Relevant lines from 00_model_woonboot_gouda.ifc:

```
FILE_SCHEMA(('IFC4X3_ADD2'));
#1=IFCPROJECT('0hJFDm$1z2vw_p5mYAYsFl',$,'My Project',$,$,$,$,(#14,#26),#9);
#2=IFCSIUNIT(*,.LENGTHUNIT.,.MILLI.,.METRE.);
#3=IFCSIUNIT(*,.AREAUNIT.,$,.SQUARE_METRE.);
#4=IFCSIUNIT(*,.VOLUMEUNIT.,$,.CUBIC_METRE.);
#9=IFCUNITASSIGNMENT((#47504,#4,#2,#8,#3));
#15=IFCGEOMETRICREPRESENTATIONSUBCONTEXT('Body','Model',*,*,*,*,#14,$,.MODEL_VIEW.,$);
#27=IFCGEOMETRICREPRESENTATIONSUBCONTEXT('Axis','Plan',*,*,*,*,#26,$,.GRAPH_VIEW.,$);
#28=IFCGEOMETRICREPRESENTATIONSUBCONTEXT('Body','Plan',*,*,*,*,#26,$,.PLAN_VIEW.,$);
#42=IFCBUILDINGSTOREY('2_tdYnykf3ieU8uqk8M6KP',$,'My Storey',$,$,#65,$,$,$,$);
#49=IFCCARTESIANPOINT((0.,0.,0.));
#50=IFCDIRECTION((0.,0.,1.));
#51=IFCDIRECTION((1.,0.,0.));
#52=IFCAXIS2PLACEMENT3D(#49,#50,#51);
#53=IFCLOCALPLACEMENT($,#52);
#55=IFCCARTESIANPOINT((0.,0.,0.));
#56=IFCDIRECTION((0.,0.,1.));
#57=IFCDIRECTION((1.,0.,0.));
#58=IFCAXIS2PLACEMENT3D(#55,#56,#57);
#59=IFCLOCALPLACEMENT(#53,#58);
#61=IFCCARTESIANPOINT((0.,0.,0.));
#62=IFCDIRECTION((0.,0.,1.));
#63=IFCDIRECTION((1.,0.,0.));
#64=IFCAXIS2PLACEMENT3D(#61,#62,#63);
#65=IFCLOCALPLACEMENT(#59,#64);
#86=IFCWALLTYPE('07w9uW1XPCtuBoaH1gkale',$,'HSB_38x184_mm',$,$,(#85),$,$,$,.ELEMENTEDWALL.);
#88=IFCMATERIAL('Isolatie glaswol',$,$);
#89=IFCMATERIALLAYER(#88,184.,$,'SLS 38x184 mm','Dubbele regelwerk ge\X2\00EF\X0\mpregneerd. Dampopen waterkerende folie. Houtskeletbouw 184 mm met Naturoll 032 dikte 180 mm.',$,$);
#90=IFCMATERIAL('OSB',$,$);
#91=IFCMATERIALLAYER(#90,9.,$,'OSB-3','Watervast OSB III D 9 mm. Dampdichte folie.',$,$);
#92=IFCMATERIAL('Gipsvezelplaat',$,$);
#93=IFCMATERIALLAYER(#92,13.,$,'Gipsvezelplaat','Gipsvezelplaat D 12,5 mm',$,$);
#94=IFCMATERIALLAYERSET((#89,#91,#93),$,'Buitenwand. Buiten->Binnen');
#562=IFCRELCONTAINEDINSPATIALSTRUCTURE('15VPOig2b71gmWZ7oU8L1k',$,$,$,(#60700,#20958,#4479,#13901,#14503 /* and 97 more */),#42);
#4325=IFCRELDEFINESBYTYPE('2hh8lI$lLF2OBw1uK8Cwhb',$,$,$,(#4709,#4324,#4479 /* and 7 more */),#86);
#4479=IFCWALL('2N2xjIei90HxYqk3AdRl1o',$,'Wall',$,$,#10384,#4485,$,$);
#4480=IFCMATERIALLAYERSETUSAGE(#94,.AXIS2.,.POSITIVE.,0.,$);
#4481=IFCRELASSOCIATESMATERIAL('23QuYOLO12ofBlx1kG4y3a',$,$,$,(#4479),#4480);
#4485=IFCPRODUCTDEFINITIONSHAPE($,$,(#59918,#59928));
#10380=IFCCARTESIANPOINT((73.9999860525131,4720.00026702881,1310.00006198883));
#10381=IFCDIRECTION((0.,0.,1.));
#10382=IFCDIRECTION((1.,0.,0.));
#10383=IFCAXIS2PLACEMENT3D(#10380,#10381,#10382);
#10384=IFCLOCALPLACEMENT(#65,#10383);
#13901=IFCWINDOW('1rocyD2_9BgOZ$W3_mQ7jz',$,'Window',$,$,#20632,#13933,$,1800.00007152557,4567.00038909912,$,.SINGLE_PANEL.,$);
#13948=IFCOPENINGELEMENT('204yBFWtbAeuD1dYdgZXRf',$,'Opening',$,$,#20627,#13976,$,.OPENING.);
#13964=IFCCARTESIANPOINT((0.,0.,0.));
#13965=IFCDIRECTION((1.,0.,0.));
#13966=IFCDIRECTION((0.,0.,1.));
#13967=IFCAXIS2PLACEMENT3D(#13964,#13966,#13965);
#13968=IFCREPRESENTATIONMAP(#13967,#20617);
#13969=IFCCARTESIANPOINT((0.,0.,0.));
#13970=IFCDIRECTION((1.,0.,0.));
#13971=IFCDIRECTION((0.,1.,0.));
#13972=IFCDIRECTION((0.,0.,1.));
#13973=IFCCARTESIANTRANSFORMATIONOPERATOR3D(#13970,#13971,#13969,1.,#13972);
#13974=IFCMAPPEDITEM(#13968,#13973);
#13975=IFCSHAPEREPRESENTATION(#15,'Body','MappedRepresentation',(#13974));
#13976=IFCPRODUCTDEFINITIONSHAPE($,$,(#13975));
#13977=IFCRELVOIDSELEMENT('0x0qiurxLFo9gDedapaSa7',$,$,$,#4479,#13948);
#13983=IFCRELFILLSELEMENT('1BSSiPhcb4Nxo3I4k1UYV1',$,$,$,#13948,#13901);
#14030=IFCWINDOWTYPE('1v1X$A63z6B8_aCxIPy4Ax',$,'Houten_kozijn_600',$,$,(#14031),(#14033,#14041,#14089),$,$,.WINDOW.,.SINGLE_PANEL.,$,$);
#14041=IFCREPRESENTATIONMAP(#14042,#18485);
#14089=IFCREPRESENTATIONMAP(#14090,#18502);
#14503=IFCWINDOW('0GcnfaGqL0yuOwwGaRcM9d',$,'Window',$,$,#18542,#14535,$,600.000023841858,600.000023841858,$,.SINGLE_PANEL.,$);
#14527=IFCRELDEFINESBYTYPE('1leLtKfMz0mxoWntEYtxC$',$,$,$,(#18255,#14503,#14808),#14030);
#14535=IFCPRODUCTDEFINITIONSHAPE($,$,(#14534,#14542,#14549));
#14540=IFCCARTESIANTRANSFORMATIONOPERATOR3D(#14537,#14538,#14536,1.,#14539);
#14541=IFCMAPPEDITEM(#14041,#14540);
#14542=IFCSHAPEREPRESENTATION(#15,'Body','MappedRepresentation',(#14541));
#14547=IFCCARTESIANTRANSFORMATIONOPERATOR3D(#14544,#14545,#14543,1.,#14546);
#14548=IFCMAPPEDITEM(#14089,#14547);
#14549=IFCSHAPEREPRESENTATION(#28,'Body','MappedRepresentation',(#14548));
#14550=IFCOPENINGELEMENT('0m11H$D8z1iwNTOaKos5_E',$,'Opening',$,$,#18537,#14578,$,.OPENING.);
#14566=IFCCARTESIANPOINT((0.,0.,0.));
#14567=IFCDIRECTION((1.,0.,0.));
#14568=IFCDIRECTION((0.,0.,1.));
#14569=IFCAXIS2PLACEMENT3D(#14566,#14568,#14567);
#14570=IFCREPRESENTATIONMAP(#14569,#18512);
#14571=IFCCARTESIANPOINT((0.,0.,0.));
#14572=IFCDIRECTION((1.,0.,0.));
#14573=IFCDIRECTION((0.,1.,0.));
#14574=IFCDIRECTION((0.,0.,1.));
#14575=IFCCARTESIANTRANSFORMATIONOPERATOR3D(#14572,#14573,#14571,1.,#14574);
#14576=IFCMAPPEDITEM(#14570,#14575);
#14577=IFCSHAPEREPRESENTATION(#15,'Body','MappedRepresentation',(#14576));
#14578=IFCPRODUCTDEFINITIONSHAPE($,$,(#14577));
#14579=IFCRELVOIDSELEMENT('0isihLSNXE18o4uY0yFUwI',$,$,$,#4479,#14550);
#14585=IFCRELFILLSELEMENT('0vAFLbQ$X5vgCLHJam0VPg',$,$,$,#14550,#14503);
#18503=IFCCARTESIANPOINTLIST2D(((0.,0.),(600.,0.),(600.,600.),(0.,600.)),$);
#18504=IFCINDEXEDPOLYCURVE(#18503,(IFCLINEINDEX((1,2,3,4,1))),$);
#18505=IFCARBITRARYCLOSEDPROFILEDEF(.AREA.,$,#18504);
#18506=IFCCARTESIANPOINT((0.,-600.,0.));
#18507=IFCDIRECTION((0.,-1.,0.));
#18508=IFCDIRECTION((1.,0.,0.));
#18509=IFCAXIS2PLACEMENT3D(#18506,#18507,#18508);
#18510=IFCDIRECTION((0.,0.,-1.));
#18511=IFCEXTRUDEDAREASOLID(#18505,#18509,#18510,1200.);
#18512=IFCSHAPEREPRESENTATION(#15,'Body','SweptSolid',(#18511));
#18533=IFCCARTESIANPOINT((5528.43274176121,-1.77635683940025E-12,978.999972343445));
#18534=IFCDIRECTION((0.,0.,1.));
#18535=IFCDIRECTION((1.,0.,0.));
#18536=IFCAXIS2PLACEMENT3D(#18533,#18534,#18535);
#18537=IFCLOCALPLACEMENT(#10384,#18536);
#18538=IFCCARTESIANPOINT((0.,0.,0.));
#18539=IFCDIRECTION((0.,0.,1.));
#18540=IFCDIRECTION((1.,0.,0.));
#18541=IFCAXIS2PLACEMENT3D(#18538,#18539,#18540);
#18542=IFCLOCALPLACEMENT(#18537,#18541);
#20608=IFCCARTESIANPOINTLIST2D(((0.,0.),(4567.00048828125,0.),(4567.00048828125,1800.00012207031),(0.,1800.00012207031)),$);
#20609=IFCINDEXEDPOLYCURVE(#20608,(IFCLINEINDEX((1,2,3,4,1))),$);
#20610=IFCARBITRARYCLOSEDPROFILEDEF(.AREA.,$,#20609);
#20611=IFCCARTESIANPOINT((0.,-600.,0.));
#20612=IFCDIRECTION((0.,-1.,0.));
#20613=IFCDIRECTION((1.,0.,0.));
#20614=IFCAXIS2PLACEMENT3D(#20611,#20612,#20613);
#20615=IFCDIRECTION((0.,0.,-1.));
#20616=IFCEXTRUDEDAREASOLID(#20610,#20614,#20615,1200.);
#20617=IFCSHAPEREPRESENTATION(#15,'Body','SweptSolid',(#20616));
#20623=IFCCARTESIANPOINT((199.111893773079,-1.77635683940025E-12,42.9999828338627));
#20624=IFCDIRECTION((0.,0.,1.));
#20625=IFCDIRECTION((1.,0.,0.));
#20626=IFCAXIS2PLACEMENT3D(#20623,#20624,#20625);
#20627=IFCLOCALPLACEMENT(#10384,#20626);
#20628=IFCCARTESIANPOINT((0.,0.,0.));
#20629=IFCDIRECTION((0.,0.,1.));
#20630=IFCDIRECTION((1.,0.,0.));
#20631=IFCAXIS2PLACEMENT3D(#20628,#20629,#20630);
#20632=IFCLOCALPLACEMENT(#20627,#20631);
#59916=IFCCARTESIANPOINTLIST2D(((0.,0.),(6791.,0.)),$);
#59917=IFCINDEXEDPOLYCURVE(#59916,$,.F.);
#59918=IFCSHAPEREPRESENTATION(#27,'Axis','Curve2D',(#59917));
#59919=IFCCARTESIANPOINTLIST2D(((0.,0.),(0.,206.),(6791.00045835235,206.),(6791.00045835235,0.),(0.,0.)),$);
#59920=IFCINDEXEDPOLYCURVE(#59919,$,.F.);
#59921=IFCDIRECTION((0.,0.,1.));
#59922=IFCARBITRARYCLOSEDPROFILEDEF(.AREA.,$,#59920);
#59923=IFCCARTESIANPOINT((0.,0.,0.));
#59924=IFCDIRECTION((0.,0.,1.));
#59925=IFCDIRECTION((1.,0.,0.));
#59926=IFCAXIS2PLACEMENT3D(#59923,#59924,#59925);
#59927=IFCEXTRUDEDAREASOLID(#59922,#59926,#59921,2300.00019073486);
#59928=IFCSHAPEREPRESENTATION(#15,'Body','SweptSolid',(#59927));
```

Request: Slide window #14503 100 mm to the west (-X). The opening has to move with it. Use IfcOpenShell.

```python
import ifcopenshell
import ifcopenshell.api.geometry
import ifcopenshell.util.placement

model = ifcopenshell.open("00_model_woonboot_gouda.ifc")

window = model.by_guid("0GcnfaGqL0yuOwwGaRcM9d")
opening = window.FillsVoids[0].RelatingOpeningElement
wall = opening.VoidsElements[0].RelatingBuildingElement

wall_matrix = ifcopenshell.util.placement.get_local_placement(wall.ObjectPlacement)
shift = wall_matrix[:3, 0] * -100.0
before = ifcopenshell.util.placement.get_local_placement(window.ObjectPlacement)[:3, 3].copy()

# The window is placed relative to its opening, so it follows when the opening moves.
matrix = ifcopenshell.util.placement.get_local_placement(opening.ObjectPlacement)
matrix[:3, 3] += shift
ifcopenshell.api.geometry.edit_object_placement(
    model, product=opening, matrix=matrix, is_si=False, should_transform_children=True
)

after = ifcopenshell.util.placement.get_local_placement(window.ObjectPlacement)[:3, 3]
print("window moved by", (after - before).round(3) + 0.0)

model.write("00_model_woonboot_gouda-out.ifc")
```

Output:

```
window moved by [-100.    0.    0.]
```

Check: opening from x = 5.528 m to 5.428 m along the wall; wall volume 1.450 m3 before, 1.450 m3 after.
